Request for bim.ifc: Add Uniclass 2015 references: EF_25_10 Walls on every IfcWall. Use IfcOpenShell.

First a look at what the model holds.

```python
import ifcopenshell

model = ifcopenshell.open("bim.ifc")
print(model.schema)
print("classifications:", [c.Name for c in model.by_type("IfcClassification")])
for ifc_class in ("IfcDoor", "IfcRoof", "IfcStair", "IfcWall", "IfcWindow"):
    print(ifc_class, len(model.by_type(ifc_class)))
```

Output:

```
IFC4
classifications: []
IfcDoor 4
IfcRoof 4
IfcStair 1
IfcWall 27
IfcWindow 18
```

```python
import ifcopenshell
import ifcopenshell.api.classification

model = ifcopenshell.open("bim.ifc")

system = ifcopenshell.api.classification.add_classification(model, classification="Uniclass 2015")

codes = {
    "IfcWall": ("EF_25_10", "Walls"),
}
for ifc_class, (code, name) in codes.items():
    products = model.by_type(ifc_class)
    ifcopenshell.api.classification.add_reference(
        model, products=products, classification=system, identification=code, name=name
    )
    print(code, len(products))

model.write("bim_rev.ifc")
```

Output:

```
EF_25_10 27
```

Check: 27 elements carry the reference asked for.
